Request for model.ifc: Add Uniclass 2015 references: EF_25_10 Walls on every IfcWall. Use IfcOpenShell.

First a look at what the model holds.

```python
import ifcopenshell

model = ifcopenshell.open("model.ifc")
print(model.schema)
print("classifications:", [c.Name for c in model.by_type("IfcClassification")])
for ifc_class in ("IfcDoor", "IfcRoof", "IfcStair", "IfcWall", "IfcWindow"):
    print(ifc_class, len(model.by_type(ifc_class)))
```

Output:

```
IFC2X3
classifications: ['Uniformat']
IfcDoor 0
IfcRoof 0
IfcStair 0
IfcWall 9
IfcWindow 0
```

```python
import ifcopenshell
import ifcopenshell.api.classification

model = ifcopenshell.open("model.ifc")

# IFC2X3 requires Source and Edition and has no link from the project to the system.
system = model.create_entity("IfcClassification", Source="NBS", Edition="2015", Name="Uniclass 2015")

codes = {
    "IfcWall": ("EF_25_10", "Walls"),
}
for ifc_class, (code, name) in codes.items():
    products = model.by_type(ifc_class)
    ifcopenshell.api.classification.add_reference(
        model, products=products, classification=system, identification=code, name=name
    )
    print(code, len(products))

model.write("model_updated.ifc")
```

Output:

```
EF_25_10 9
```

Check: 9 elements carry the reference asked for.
